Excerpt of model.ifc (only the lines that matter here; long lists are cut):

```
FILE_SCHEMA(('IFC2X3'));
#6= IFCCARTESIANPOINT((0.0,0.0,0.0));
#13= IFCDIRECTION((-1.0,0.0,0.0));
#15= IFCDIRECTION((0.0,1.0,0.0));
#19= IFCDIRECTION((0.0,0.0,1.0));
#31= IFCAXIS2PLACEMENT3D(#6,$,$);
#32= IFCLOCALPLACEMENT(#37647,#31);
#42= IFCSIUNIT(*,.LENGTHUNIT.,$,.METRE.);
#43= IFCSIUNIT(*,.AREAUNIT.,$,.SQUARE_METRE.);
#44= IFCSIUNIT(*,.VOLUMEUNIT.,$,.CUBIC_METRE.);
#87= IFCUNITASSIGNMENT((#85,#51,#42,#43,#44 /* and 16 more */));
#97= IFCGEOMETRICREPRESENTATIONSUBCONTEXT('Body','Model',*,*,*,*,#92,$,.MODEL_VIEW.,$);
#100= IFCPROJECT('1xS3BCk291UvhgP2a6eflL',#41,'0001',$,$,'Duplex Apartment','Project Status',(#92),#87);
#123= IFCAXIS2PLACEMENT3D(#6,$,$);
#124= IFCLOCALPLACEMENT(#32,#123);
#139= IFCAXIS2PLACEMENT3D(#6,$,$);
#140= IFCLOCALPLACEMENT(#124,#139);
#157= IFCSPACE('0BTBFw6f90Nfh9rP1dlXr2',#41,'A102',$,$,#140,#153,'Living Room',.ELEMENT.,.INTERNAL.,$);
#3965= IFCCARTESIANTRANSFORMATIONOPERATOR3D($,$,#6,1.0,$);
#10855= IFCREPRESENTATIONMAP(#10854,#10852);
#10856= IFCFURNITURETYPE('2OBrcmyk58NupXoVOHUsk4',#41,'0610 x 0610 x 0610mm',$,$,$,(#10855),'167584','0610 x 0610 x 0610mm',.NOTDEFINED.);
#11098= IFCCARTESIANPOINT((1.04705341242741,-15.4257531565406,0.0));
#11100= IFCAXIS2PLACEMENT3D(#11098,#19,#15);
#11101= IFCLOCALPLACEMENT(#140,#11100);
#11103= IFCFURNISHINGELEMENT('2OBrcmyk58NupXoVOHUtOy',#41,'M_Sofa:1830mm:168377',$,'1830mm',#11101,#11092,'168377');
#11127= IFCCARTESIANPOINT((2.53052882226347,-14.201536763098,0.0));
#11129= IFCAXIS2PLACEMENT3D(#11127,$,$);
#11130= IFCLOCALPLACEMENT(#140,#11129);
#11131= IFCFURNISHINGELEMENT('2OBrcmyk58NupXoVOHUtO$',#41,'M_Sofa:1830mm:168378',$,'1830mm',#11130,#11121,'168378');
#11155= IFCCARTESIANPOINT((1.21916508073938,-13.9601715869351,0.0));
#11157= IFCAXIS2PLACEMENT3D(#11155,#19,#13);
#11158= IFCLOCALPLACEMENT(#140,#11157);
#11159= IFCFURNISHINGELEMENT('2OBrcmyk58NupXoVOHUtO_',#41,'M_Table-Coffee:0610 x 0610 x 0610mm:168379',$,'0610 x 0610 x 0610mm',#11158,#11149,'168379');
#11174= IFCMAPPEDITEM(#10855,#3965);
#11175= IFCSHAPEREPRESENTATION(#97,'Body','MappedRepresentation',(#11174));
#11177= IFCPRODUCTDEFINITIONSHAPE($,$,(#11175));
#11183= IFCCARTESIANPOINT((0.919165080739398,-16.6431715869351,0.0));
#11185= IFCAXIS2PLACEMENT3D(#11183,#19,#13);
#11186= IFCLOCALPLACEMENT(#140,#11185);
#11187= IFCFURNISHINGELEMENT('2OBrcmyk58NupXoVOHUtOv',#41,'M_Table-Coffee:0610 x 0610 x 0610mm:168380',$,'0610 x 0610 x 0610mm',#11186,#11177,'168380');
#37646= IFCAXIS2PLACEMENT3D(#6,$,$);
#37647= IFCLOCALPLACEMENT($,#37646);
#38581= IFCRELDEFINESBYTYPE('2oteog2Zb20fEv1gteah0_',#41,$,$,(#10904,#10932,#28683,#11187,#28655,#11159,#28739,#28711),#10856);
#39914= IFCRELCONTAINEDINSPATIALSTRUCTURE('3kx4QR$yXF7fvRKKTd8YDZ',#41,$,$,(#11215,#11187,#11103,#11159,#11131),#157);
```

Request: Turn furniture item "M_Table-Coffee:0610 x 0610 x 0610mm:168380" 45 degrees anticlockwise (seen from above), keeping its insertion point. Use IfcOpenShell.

```python
import ifcopenshell
import ifcopenshell.api.geometry
import ifcopenshell.util.placement

model = ifcopenshell.open("model.ifc")

item = model.by_id(11187)
matrix = ifcopenshell.util.placement.get_local_placement(item.ObjectPlacement)
matrix = matrix @ ifcopenshell.util.placement.rotation(45, "Z")
ifcopenshell.api.geometry.edit_object_placement(model, product=item, matrix=matrix, is_si=False)

print(ifcopenshell.util.placement.get_local_placement(item.ObjectPlacement).round(3) + 0.0)

model.write("model_updated.ifc")
```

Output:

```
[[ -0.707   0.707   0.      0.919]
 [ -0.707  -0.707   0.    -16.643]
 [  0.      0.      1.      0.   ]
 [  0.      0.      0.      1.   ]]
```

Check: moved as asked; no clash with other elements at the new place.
